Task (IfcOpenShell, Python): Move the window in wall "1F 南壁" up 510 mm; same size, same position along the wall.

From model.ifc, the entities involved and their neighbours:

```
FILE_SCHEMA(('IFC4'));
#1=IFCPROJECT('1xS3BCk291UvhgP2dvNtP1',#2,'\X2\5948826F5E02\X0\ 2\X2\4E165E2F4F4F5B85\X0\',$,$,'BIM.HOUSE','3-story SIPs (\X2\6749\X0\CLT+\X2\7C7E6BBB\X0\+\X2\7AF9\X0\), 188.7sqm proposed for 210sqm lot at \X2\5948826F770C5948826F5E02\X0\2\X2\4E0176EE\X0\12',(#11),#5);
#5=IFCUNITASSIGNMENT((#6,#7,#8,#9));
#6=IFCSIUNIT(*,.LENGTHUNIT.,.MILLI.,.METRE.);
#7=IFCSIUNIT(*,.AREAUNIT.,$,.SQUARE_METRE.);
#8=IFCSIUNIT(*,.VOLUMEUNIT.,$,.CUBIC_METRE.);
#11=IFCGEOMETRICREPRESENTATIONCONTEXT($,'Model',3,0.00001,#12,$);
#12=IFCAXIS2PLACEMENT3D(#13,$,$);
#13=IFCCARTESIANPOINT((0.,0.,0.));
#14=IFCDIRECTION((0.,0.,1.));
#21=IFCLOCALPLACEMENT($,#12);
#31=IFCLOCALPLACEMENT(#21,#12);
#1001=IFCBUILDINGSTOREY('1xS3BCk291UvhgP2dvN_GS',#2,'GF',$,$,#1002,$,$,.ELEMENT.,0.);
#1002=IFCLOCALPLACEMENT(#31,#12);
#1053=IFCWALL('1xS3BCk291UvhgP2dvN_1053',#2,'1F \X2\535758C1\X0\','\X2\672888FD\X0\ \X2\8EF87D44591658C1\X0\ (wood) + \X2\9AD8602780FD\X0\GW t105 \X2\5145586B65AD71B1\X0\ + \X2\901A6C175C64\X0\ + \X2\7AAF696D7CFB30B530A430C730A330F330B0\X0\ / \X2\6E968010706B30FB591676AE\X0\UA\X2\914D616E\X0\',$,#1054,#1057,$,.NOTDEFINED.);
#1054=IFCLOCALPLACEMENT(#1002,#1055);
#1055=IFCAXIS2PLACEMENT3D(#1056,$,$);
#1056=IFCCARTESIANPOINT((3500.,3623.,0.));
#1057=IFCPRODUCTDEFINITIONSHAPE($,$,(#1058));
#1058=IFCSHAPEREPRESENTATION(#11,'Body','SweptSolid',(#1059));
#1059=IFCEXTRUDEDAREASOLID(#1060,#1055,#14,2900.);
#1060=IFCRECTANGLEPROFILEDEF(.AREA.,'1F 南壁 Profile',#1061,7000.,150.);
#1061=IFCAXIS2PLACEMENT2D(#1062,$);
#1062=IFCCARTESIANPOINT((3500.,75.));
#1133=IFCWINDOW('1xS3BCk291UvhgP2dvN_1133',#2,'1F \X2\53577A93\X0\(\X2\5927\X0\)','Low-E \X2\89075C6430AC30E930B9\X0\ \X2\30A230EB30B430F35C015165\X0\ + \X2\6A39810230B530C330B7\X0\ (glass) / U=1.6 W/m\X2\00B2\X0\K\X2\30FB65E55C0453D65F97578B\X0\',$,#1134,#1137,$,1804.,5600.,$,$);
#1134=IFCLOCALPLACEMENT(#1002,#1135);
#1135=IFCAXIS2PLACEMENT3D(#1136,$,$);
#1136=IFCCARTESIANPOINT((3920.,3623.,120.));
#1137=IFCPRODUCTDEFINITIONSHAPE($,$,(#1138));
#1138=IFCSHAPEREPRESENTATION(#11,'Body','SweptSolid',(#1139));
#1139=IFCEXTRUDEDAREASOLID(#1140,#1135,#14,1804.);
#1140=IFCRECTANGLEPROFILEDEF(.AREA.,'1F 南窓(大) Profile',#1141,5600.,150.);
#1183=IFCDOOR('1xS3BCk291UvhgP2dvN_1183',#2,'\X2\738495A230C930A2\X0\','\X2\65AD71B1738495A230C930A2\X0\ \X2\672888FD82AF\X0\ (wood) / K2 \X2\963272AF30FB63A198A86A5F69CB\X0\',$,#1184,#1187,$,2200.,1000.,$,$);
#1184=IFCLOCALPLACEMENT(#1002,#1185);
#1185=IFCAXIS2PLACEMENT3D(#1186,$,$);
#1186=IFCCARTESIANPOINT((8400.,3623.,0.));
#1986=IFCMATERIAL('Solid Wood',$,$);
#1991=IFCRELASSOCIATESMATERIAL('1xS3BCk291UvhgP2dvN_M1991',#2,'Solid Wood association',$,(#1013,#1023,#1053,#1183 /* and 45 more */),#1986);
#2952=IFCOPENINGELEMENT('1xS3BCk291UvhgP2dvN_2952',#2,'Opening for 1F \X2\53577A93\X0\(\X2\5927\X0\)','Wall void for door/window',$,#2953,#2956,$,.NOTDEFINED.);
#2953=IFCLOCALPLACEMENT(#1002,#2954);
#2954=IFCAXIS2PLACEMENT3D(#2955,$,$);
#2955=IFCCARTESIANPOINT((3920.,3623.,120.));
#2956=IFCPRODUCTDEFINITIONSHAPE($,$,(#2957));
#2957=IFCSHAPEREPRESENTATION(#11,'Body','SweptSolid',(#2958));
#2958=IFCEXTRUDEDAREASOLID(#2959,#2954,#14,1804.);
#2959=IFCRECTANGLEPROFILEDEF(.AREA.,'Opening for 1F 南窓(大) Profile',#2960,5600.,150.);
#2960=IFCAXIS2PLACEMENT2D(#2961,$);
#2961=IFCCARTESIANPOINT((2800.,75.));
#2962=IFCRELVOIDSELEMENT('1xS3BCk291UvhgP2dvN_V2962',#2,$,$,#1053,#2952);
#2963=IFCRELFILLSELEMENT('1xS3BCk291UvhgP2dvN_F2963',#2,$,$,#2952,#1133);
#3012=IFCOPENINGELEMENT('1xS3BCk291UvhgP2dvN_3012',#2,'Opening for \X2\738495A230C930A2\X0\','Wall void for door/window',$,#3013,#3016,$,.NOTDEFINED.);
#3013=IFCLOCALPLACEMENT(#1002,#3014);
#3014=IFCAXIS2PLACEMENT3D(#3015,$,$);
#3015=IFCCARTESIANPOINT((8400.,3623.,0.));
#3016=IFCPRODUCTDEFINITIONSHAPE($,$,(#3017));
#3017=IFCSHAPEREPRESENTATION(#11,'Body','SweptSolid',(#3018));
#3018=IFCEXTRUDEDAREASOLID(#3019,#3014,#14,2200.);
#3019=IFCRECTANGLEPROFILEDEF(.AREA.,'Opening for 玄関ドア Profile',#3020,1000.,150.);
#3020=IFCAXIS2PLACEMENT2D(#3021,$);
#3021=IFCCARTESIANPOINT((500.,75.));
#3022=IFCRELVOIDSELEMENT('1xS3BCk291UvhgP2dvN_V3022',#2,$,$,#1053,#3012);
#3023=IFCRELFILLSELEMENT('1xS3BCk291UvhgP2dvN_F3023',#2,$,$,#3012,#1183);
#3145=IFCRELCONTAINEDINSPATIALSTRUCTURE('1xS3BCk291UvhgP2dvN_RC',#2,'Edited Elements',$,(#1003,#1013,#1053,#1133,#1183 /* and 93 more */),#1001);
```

```python
import numpy as np
import ifcopenshell
import ifcopenshell.api.geometry
import ifcopenshell.util.placement
import ifcopenshell.util.unit

model = ifcopenshell.open("model.ifc")
unit_scale = ifcopenshell.util.unit.calculate_unit_scale(model)

window = model.by_guid("1xS3BCk291UvhgP2dvN_1133")
opening = window.FillsVoids[0].RelatingOpeningElement
dz = 0.51 / unit_scale

shift = np.array([0.0, 0.0, dz])
# The window is not placed relative to its opening, so move both.
for product in (opening, window):
    matrix = ifcopenshell.util.placement.get_local_placement(product.ObjectPlacement)
    matrix[:3, 3] += shift
    ifcopenshell.api.geometry.edit_object_placement(model, product=product, matrix=matrix, is_si=False)

print(f"moved by {dz * unit_scale:+.3f} m")

model.write("model-out.ifc")
```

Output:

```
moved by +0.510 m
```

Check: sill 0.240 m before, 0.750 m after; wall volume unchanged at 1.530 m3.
